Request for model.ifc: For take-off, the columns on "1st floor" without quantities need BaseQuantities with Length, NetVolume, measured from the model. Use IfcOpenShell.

First a look at what the model holds.

```python
import ifcopenshell
import ifcopenshell.util.element
import ifcopenshell.util.unit

model = ifcopenshell.open("model.ifc")
print(model.schema)
for unit_type in ("LENGTHUNIT", "AREAUNIT", "VOLUMEUNIT"):
    print(unit_type, ifcopenshell.util.unit.calculate_unit_scale(model, unit_type))
storey = next(s for s in model.by_type("IfcBuildingStorey") if s.Name == "1st floor")
columns = [e for e in ifcopenshell.util.element.get_decomposition(storey) if e.is_a("IfcColumn")]
for e in sorted(columns, key=lambda e: e.id()):
    print(e.id(), e.is_a(), e.Name, list(ifcopenshell.util.element.get_psets(e, qtos_only=True)), sep=" | ")
```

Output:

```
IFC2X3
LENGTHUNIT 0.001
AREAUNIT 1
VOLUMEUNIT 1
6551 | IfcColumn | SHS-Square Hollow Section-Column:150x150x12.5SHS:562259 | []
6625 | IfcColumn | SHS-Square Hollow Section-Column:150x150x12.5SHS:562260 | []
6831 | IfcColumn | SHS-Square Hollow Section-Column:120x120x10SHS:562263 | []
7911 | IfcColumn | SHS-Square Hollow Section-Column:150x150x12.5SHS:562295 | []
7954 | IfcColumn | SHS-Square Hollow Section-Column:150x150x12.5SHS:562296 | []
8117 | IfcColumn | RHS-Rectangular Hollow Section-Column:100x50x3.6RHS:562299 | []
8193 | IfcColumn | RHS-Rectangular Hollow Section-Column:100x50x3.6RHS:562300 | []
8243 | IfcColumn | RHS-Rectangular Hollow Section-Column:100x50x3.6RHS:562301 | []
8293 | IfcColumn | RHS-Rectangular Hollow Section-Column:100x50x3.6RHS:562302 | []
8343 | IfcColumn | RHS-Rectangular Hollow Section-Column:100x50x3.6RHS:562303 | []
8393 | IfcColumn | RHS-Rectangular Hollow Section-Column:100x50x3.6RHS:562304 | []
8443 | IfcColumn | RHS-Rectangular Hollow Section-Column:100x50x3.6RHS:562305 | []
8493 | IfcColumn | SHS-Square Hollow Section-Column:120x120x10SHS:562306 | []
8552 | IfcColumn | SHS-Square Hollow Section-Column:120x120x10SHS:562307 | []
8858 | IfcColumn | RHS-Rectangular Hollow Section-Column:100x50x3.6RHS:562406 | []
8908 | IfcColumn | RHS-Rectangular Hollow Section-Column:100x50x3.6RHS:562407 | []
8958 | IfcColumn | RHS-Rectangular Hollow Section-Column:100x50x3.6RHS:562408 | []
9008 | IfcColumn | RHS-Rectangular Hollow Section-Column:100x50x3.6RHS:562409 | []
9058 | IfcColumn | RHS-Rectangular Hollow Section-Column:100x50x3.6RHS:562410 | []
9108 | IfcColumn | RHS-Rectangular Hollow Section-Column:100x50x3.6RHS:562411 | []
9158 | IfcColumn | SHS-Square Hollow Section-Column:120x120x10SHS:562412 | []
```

```python
import ifcopenshell
import ifcopenshell.api.pset
import ifcopenshell.geom
import ifcopenshell.util.element
import ifcopenshell.util.shape
import ifcopenshell.util.unit

model = ifcopenshell.open("model.ifc")
unit_scale = ifcopenshell.util.unit.calculate_unit_scale(model)
volume_scale = ifcopenshell.util.unit.calculate_unit_scale(model, "VOLUMEUNIT")
settings = ifcopenshell.geom.settings()

storey = next(s for s in model.by_type("IfcBuildingStorey") if s.Name == "1st floor")
columns = [e for e in ifcopenshell.util.element.get_decomposition(storey) if e.is_a("IfcColumn")]

for e in sorted(columns, key=lambda e: e.id()):
    if ifcopenshell.util.element.get_psets(e, qtos_only=True, should_inherit=False):
        continue
    # Geometry comes back in metres, in the element's own axes.
    shape = ifcopenshell.geom.create_shape(settings, e)
    values = {
        "Length": ifcopenshell.util.shape.get_z(shape.geometry) / unit_scale,
        "NetVolume": ifcopenshell.util.shape.get_volume(shape.geometry) / volume_scale,
    }
    qto = ifcopenshell.api.pset.add_qto(model, product=e, name="BaseQuantities")
    ifcopenshell.api.pset.edit_qto(model, qto=qto, properties=values)
    print(e.id(), {k: round(v, 3) for k, v in values.items()})

model.write("model-out.ifc")
```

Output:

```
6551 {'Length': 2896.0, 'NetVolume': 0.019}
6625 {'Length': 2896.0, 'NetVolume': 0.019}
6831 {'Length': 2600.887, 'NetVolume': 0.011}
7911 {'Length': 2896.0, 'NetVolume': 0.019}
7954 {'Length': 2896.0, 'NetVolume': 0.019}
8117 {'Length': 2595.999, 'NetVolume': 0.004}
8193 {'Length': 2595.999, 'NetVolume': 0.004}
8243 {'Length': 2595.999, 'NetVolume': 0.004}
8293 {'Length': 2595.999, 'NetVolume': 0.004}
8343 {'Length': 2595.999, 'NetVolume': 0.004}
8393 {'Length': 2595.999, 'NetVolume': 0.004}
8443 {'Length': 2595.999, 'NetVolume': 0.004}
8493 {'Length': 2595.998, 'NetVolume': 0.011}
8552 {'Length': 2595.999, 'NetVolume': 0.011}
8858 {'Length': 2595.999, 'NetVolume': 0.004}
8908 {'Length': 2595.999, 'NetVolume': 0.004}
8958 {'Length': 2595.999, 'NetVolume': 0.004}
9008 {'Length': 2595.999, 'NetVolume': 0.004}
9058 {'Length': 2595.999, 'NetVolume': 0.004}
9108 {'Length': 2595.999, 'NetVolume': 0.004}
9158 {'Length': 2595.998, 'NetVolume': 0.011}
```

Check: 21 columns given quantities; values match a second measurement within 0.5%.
